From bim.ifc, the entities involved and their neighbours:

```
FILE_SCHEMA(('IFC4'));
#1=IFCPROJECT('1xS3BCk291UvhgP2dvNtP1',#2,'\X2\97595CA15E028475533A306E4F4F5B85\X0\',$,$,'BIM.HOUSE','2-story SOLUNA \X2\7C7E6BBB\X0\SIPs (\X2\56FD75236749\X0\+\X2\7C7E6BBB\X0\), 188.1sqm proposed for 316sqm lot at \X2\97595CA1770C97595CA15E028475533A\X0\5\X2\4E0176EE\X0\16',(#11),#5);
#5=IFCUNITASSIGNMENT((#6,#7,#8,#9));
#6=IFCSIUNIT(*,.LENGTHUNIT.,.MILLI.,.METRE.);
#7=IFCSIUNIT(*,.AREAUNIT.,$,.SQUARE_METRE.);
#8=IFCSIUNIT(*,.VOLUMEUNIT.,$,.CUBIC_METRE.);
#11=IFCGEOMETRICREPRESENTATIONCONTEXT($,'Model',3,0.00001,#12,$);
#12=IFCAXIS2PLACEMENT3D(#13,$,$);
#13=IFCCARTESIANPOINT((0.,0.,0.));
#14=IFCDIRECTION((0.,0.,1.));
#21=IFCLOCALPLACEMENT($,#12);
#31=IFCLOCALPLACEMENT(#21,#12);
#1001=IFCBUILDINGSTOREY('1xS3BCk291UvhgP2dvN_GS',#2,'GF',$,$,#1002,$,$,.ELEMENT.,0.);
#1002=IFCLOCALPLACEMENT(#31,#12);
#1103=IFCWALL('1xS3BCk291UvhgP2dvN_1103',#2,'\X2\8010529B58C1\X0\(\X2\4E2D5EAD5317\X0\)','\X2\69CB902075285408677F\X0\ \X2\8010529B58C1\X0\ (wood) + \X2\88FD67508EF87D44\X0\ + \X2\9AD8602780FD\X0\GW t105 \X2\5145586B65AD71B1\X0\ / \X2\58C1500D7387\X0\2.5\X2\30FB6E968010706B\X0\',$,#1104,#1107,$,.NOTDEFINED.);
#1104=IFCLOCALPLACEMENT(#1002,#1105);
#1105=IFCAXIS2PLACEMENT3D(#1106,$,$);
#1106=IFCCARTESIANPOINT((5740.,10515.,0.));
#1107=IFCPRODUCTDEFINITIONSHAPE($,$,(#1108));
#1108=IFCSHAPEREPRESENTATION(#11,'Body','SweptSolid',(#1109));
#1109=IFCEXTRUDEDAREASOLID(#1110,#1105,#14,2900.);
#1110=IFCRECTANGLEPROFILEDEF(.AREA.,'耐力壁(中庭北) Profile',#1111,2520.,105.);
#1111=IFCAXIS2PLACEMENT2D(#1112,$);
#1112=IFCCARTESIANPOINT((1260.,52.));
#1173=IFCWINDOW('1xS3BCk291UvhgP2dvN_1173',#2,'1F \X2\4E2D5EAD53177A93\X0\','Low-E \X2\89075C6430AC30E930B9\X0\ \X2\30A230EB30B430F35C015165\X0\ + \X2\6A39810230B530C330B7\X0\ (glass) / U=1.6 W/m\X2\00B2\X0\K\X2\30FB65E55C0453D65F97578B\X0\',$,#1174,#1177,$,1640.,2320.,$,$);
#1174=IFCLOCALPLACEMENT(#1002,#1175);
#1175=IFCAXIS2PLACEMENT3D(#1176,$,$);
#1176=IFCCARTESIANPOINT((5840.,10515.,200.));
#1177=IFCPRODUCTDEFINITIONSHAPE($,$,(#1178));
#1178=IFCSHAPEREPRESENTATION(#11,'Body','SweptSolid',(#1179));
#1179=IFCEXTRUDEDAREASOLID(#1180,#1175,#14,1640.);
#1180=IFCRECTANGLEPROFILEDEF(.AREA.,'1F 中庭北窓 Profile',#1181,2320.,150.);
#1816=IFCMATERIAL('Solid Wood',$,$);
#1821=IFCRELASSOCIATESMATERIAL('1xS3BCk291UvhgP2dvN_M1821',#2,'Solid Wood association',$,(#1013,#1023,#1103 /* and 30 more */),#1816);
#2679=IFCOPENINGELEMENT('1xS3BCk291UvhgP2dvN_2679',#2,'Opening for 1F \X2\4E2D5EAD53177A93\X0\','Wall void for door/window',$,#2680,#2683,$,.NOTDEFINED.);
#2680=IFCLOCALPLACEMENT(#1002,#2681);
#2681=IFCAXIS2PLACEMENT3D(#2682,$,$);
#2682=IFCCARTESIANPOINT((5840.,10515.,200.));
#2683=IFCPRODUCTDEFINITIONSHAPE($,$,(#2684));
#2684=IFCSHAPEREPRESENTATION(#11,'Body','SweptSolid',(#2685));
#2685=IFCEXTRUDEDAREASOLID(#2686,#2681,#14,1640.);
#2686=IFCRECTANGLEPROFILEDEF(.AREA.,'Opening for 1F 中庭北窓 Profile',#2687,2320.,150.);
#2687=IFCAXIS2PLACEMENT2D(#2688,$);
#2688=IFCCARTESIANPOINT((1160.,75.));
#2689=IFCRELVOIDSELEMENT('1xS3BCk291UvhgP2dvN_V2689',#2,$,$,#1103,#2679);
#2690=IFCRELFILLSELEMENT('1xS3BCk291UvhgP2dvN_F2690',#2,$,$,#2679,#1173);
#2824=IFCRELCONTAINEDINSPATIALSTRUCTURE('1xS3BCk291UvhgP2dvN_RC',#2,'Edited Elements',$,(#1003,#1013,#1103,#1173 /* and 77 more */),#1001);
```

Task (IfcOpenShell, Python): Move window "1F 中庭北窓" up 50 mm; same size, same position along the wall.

```python
import numpy as np
import ifcopenshell
import ifcopenshell.api.geometry
import ifcopenshell.util.placement
import ifcopenshell.util.unit

model = ifcopenshell.open("bim.ifc")
unit_scale = ifcopenshell.util.unit.calculate_unit_scale(model)

window = model.by_guid("1xS3BCk291UvhgP2dvN_1173")
opening = window.FillsVoids[0].RelatingOpeningElement
dz = 0.05 / unit_scale

shift = np.array([0.0, 0.0, dz])
# The window is not placed relative to its opening, so move both.
for product in (opening, window):
    matrix = ifcopenshell.util.placement.get_local_placement(product.ObjectPlacement)
    matrix[:3, 3] += shift
    ifcopenshell.api.geometry.edit_object_placement(model, product=product, matrix=matrix, is_si=False)

print(f"moved by {dz * unit_scale:+.3f} m")

model.write("bim_edited.ifc")
```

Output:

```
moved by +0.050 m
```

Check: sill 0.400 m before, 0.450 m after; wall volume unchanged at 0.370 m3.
